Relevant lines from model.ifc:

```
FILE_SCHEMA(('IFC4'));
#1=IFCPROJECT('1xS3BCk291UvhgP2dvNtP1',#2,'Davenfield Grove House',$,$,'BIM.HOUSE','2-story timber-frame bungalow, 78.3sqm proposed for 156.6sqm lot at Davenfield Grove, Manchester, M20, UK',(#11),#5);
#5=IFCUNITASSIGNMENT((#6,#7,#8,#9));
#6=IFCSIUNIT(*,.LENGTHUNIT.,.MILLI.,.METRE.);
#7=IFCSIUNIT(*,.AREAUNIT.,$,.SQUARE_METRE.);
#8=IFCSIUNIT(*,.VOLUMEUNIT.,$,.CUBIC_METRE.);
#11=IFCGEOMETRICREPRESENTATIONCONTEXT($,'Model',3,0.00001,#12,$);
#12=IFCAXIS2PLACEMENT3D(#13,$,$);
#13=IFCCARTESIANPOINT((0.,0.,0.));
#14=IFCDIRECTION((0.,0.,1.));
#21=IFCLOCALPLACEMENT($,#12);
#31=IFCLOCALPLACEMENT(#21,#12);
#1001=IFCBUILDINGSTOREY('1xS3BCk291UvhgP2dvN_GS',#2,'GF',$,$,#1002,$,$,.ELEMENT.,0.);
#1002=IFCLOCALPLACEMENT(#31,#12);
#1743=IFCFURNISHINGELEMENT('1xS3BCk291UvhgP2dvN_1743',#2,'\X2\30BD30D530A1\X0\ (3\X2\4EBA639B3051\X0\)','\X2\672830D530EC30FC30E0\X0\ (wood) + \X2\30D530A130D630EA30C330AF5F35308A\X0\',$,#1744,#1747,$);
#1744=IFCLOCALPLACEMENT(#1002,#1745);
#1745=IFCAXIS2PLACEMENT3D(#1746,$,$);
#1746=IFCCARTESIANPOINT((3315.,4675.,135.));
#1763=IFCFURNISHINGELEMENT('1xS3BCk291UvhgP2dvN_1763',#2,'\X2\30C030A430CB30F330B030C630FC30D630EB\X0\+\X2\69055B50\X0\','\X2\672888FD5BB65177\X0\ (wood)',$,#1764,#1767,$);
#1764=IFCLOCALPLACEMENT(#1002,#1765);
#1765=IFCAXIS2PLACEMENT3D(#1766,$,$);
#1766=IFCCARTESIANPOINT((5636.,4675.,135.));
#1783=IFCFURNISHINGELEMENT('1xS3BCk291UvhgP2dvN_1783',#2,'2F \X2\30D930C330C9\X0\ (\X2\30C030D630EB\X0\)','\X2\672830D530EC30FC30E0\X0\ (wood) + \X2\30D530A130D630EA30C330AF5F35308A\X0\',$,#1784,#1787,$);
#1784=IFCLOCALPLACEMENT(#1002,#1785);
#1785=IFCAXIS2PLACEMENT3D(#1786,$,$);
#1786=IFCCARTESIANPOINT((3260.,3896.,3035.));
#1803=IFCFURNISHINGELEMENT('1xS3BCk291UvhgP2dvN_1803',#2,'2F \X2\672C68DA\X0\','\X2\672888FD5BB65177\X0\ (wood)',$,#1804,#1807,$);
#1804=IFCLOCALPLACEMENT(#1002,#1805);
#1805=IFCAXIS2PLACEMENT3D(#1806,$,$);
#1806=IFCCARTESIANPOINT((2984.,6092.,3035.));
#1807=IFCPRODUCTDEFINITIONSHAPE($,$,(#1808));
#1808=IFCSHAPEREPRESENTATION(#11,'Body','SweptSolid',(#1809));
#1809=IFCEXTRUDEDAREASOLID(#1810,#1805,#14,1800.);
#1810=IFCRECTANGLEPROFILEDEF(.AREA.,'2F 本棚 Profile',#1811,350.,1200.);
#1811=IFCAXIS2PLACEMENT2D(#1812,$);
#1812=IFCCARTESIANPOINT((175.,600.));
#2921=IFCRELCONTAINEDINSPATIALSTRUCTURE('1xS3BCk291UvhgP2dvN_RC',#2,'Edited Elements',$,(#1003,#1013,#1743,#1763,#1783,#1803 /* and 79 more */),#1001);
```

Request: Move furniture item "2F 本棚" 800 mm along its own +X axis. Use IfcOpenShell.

```python
import ifcopenshell
import ifcopenshell.api.geometry
import ifcopenshell.util.placement

model = ifcopenshell.open("model.ifc")

item = model.by_guid("1xS3BCk291UvhgP2dvN_1803")
matrix = ifcopenshell.util.placement.get_local_placement(item.ObjectPlacement)
matrix[:3, 3] += matrix[:3, 0] * 800.0
ifcopenshell.api.geometry.edit_object_placement(model, product=item, matrix=matrix, is_si=False)

print(ifcopenshell.util.placement.get_local_placement(item.ObjectPlacement).round(3) + 0.0)

model.write("model-out.ifc")
```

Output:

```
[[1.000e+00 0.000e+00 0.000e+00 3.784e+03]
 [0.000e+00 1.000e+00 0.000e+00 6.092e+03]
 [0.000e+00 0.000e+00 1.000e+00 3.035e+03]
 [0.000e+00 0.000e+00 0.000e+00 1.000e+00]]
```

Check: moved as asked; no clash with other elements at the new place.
